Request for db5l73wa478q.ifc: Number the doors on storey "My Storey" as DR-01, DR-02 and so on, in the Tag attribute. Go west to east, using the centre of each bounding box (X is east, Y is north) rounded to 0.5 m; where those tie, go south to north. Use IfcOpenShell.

First a look at what the model holds.

```python
import ifcopenshell
import ifcopenshell.util.element
import ifcopenshell.util.placement

model = ifcopenshell.open("db5l73wa478q.ifc")
print(model.schema)
storey = next(s for s in model.by_type("IfcBuildingStorey") if s.Name == "My Storey")
doors = [e for e in ifcopenshell.util.element.get_decomposition(storey) if e.is_a("IfcDoor")]
for e in sorted(doors, key=lambda e: e.id()):
    origin = ifcopenshell.util.placement.get_local_placement(e.ObjectPlacement)[:3, 3]
    print(e.id(), e.Tag, e.Name, origin.round(2) + 0.0, sep=" | ")
```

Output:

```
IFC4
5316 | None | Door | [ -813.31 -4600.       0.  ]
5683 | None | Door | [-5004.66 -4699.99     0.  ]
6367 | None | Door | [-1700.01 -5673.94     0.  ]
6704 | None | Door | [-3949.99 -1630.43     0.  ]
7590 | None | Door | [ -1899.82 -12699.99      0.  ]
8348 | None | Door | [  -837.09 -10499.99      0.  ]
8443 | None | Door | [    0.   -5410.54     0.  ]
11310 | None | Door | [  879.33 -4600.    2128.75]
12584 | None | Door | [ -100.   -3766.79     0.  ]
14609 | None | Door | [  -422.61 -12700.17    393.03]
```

```python
import ifcopenshell
import ifcopenshell.geom
import ifcopenshell.util.element
import ifcopenshell.util.shape

model = ifcopenshell.open("db5l73wa478q.ifc")
settings = ifcopenshell.geom.settings()
settings.set("use-world-coords", True)


def centre(element):
    shape = ifcopenshell.geom.create_shape(settings, element)
    return ifcopenshell.util.shape.get_bbox_centroid(shape.geometry)


storey = next(s for s in model.by_type("IfcBuildingStorey") if s.Name == "My Storey")
doors = [e for e in ifcopenshell.util.element.get_decomposition(storey) if e.is_a("IfcDoor")]

# Insertion points can sit at a corner or the storey origin, so sort by the geometry (in metres).
centres = {e: centre(e) for e in doors}
doors.sort(key=lambda e: (round(centres[e][0] / 0.5), centres[e][1]))

for i, e in enumerate(doors, start=1):
    number = f"DR-{i:02d}"
    e.Tag = number
    print(e.id(), number)

model.write("db5l73wa478q_v2.ifc")
```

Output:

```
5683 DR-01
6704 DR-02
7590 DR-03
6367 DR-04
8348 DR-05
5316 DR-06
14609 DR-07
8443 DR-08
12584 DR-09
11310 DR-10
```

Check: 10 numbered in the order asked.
